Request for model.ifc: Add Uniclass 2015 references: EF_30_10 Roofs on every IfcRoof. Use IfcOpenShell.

First a look at what the model holds.

```python
import ifcopenshell

model = ifcopenshell.open("model.ifc")
print(model.schema)
print("classifications:", [c.Name for c in model.by_type("IfcClassification")])
for ifc_class in ("IfcDoor", "IfcRoof", "IfcStair", "IfcWall", "IfcWindow"):
    print(ifc_class, len(model.by_type(ifc_class)))
```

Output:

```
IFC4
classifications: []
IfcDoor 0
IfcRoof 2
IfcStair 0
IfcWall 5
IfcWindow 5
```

```python
import ifcopenshell
import ifcopenshell.api.classification

model = ifcopenshell.open("model.ifc")

system = ifcopenshell.api.classification.add_classification(model, classification="Uniclass 2015")

codes = {
    "IfcRoof": ("EF_30_10", "Roofs"),
}
for ifc_class, (code, name) in codes.items():
    products = model.by_type(ifc_class)
    ifcopenshell.api.classification.add_reference(
        model, products=products, classification=system, identification=code, name=name
    )
    print(code, len(products))

model.write("model-out.ifc")
```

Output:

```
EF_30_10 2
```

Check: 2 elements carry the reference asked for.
